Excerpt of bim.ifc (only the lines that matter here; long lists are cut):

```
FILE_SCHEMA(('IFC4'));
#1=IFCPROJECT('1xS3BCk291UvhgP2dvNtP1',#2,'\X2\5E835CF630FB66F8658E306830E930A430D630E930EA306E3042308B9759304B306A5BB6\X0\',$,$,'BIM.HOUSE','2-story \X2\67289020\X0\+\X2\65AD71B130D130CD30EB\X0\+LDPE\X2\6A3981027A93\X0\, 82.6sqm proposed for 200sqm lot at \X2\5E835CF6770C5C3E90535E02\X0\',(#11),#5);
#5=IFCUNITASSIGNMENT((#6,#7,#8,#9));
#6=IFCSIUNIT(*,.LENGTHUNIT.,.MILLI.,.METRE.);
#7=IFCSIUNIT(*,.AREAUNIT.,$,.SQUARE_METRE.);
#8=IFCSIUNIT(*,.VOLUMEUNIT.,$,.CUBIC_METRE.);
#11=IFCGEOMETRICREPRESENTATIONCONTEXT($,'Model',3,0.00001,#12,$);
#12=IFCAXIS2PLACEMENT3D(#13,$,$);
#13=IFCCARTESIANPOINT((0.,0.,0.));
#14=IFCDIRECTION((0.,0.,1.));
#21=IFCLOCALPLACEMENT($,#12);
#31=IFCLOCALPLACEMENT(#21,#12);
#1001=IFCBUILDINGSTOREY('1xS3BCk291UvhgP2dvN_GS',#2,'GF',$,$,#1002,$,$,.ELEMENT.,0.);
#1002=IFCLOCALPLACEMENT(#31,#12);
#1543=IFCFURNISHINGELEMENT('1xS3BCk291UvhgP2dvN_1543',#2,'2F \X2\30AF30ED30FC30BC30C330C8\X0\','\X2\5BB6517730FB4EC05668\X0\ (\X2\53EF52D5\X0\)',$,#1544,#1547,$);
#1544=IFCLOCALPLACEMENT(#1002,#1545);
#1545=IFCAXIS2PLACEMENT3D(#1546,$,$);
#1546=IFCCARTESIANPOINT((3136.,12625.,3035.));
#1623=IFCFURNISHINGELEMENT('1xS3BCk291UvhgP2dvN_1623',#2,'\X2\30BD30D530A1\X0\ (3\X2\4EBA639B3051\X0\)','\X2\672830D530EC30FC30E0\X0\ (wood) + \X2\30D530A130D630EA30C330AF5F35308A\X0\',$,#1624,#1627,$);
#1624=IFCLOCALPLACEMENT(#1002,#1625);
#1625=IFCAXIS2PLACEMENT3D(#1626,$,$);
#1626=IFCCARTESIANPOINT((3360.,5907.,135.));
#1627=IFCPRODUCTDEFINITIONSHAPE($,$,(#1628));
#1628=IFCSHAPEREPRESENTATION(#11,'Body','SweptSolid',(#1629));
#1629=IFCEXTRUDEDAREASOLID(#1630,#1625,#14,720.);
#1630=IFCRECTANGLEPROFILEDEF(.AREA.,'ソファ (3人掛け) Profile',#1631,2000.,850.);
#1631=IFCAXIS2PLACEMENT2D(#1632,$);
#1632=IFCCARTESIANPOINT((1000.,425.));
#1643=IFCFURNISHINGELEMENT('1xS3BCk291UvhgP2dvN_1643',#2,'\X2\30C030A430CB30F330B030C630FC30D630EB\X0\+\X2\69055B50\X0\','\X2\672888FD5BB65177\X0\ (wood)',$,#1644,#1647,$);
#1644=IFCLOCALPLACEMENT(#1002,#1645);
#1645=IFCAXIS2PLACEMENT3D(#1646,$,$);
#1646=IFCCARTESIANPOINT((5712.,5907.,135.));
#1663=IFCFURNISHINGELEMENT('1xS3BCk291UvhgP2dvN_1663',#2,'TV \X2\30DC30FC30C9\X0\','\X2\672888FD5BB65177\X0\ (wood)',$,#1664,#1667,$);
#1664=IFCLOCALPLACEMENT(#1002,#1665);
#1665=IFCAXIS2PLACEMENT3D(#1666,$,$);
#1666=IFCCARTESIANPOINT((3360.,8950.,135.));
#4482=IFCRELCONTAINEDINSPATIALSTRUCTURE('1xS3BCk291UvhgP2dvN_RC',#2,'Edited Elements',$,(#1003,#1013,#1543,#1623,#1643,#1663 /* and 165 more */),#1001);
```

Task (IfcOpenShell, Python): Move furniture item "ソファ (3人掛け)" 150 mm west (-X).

```python
import ifcopenshell
import ifcopenshell.api.geometry
import ifcopenshell.util.placement
import ifcopenshell.util.unit

model = ifcopenshell.open("bim.ifc")
unit_scale = ifcopenshell.util.unit.calculate_unit_scale(model)

item = model.by_id(1623)
matrix = ifcopenshell.util.placement.get_local_placement(item.ObjectPlacement)
matrix[0, 3] -= 0.15 / unit_scale
ifcopenshell.api.geometry.edit_object_placement(model, product=item, matrix=matrix, is_si=False)

print(ifcopenshell.util.placement.get_local_placement(item.ObjectPlacement).round(3) + 0.0)

model.write("bim_rev.ifc")
```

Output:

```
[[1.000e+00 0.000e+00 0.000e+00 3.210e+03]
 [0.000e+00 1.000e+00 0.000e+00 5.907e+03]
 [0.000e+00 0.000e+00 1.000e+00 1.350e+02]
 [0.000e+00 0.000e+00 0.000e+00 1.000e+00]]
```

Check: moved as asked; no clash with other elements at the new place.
